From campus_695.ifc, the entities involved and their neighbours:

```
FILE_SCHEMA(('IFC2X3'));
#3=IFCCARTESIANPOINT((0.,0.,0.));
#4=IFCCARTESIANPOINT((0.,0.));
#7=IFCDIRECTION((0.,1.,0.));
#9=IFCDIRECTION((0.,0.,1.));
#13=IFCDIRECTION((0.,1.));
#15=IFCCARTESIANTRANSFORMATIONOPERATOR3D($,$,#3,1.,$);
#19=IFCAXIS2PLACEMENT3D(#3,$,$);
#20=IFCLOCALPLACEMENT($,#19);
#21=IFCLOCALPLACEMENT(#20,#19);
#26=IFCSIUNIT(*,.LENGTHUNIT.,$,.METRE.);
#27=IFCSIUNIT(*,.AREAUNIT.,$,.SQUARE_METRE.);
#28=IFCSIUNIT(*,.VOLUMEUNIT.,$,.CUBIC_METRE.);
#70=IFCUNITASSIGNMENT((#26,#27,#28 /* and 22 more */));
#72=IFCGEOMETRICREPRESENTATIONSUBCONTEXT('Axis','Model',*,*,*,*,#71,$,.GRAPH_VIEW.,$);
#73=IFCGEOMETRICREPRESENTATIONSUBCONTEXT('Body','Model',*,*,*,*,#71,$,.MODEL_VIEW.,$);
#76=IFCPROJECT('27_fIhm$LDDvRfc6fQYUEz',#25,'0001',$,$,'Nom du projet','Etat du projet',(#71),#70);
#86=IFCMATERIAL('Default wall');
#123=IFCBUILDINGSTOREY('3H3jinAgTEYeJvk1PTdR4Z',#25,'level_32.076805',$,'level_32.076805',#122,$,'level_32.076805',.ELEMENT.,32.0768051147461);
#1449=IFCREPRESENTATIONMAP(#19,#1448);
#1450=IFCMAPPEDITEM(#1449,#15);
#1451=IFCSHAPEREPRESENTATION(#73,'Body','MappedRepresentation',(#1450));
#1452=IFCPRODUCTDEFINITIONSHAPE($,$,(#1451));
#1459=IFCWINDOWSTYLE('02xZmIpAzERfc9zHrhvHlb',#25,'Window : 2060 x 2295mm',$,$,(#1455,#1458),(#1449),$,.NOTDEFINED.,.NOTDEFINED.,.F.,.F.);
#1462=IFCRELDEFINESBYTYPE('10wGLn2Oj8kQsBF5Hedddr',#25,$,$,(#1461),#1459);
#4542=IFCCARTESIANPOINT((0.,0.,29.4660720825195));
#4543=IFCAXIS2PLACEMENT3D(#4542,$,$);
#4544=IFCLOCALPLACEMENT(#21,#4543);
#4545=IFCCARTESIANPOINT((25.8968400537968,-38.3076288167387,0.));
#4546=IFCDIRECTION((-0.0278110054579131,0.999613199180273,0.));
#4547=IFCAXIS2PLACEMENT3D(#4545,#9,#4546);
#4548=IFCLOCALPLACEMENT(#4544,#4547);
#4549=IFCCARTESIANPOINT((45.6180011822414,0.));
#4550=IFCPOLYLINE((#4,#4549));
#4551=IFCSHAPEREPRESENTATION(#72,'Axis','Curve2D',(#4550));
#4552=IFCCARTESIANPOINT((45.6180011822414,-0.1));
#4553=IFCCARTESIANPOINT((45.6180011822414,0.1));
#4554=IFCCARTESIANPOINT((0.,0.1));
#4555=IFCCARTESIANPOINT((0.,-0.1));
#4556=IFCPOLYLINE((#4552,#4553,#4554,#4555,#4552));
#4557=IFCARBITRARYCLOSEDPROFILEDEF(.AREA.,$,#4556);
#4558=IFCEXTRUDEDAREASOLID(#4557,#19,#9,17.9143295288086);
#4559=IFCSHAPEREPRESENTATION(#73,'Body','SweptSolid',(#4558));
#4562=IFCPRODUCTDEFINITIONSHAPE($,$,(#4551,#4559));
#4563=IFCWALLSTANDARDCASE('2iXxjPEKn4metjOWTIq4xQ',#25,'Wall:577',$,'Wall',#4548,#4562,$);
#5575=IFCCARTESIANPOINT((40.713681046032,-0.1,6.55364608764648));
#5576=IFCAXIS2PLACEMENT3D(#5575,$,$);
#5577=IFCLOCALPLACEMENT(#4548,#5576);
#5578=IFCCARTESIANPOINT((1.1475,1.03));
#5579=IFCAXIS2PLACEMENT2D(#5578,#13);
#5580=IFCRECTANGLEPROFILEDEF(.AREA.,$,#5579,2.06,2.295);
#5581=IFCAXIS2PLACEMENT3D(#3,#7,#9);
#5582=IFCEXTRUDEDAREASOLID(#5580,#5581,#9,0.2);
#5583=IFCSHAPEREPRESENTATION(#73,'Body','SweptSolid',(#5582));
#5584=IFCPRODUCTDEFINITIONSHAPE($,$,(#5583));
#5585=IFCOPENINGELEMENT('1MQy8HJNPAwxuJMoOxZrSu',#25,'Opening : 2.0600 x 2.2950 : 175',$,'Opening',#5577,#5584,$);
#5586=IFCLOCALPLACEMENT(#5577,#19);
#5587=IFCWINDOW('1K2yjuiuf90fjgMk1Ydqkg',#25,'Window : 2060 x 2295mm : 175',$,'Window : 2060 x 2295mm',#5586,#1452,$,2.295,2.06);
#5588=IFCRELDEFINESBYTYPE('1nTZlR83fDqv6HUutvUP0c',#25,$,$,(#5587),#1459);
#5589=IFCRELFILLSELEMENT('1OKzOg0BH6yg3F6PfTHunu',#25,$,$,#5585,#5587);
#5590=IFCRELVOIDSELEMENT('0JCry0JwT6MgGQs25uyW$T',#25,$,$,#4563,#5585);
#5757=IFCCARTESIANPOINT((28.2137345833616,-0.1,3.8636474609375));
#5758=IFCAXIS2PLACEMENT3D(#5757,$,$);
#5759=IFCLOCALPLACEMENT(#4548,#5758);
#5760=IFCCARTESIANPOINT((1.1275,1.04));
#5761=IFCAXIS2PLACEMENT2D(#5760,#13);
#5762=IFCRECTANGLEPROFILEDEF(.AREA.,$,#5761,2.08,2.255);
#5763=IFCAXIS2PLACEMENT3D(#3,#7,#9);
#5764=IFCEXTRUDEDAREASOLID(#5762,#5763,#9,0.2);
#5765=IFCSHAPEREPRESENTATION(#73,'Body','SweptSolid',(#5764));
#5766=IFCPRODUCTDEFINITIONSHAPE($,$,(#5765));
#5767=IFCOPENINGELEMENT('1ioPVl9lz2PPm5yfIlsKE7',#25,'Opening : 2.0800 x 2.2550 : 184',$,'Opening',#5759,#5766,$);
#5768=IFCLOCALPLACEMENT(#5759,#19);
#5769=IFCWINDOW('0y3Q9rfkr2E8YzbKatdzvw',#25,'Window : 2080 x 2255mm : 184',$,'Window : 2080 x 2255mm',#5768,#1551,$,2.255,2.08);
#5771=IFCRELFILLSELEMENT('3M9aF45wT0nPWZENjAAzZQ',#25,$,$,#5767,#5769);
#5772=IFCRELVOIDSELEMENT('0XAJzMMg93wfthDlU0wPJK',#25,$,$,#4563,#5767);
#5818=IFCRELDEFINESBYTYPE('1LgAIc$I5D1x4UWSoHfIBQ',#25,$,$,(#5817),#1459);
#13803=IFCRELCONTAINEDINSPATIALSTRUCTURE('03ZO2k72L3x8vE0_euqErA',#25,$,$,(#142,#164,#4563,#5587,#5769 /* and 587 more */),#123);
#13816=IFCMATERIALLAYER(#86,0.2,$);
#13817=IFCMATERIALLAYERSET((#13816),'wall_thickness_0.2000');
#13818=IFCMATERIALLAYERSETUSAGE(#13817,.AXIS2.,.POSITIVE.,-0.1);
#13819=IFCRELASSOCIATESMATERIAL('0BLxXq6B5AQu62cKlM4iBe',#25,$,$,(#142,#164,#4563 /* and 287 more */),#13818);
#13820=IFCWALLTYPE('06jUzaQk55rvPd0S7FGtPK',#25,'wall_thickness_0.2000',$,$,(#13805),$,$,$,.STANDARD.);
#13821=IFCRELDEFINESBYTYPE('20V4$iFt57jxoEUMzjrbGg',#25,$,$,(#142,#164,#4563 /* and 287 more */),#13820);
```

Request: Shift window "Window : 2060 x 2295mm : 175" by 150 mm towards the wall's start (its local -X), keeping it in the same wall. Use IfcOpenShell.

```python
import ifcopenshell
import ifcopenshell.api.geometry
import ifcopenshell.util.placement
import ifcopenshell.util.unit

model = ifcopenshell.open("campus_695.ifc")
unit_scale = ifcopenshell.util.unit.calculate_unit_scale(model)

window = model.by_guid("1K2yjuiuf90fjgMk1Ydqkg")
opening = window.FillsVoids[0].RelatingOpeningElement
wall = opening.VoidsElements[0].RelatingBuildingElement

wall_matrix = ifcopenshell.util.placement.get_local_placement(wall.ObjectPlacement)
shift = wall_matrix[:3, 0] * -0.15 / unit_scale
before = ifcopenshell.util.placement.get_local_placement(window.ObjectPlacement)[:3, 3].copy()

# The window is placed relative to its opening, so it follows when the opening moves.
matrix = ifcopenshell.util.placement.get_local_placement(opening.ObjectPlacement)
matrix[:3, 3] += shift
ifcopenshell.api.geometry.edit_object_placement(
    model, product=opening, matrix=matrix, is_si=False, should_transform_children=True
)

after = ifcopenshell.util.placement.get_local_placement(window.ObjectPlacement)[:3, 3]
print("window moved by", (after - before).round(3) + 0.0)

model.write("campus_695_rev.ifc")
```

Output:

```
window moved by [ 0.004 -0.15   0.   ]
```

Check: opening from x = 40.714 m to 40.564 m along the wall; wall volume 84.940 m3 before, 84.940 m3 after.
